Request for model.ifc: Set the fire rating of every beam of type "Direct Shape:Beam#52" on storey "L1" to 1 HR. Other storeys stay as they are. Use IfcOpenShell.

First a look at what the model holds.

```python
import ifcopenshell
import ifcopenshell.util.element

model = ifcopenshell.open("model.ifc")
print(model.schema)
storey = next(s for s in model.by_type("IfcBuildingStorey") if s.Name == "L1")
beams = [e for e in ifcopenshell.util.element.get_decomposition(storey) if e.is_a("IfcBeam")]
seen = {}
for e in beams:
    element_type = ifcopenshell.util.element.get_type(e)
    key = (element_type.Name if element_type != e and element_type else None, ifcopenshell.util.element.get_pset(e, "Pset_BeamCommon", "FireRating"))
    seen[key] = seen.get(key, 0) + 1
for (name, value), count in sorted(seen.items(), key=str):
    print(count, "x", name, "|", value)
```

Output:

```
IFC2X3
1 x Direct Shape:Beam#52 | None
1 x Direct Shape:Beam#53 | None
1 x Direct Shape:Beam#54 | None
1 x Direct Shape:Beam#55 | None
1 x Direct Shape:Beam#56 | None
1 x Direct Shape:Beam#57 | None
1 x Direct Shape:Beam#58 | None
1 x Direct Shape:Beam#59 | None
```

```python
import ifcopenshell
import ifcopenshell.api.pset
import ifcopenshell.util.element

model = ifcopenshell.open("model.ifc")

storey = next(s for s in model.by_type("IfcBuildingStorey") if s.Name == "L1")
beams = [e for e in ifcopenshell.util.element.get_decomposition(storey) if e.is_a("IfcBeam")]

count = 0
for e in beams:
    element_type = ifcopenshell.util.element.get_type(e)
    if element_type in (None, e) or element_type.Name != "Direct Shape:Beam#52":
        continue
    # add_pset returns the element's existing set when there is one.
    pset = ifcopenshell.api.pset.add_pset(model, product=e, name="Pset_BeamCommon")
    ifcopenshell.api.pset.edit_pset(model, pset=pset, properties={"FireRating": "1 HR"})
    count += 1

print(count, "beams updated")

model.write("model_rev.ifc")
```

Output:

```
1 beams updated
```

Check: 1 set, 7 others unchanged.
